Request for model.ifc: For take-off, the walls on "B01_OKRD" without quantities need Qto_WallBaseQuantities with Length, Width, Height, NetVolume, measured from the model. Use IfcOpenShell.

First a look at what the model holds.

```python
import ifcopenshell
import ifcopenshell.util.element
import ifcopenshell.util.unit

model = ifcopenshell.open("model.ifc")
print(model.schema)
for unit_type in ("LENGTHUNIT", "AREAUNIT", "VOLUMEUNIT"):
    print(unit_type, ifcopenshell.util.unit.calculate_unit_scale(model, unit_type))
storey = next(s for s in model.by_type("IfcBuildingStorey") if s.Name == "B01_OKRD")
walls = [e for e in ifcopenshell.util.element.get_decomposition(storey) if e.is_a("IfcWall")]
for e in sorted(walls, key=lambda e: e.id()):
    print(e.id(), e.is_a(), e.Name, list(ifcopenshell.util.element.get_psets(e, qtos_only=True)), sep=" | ")
```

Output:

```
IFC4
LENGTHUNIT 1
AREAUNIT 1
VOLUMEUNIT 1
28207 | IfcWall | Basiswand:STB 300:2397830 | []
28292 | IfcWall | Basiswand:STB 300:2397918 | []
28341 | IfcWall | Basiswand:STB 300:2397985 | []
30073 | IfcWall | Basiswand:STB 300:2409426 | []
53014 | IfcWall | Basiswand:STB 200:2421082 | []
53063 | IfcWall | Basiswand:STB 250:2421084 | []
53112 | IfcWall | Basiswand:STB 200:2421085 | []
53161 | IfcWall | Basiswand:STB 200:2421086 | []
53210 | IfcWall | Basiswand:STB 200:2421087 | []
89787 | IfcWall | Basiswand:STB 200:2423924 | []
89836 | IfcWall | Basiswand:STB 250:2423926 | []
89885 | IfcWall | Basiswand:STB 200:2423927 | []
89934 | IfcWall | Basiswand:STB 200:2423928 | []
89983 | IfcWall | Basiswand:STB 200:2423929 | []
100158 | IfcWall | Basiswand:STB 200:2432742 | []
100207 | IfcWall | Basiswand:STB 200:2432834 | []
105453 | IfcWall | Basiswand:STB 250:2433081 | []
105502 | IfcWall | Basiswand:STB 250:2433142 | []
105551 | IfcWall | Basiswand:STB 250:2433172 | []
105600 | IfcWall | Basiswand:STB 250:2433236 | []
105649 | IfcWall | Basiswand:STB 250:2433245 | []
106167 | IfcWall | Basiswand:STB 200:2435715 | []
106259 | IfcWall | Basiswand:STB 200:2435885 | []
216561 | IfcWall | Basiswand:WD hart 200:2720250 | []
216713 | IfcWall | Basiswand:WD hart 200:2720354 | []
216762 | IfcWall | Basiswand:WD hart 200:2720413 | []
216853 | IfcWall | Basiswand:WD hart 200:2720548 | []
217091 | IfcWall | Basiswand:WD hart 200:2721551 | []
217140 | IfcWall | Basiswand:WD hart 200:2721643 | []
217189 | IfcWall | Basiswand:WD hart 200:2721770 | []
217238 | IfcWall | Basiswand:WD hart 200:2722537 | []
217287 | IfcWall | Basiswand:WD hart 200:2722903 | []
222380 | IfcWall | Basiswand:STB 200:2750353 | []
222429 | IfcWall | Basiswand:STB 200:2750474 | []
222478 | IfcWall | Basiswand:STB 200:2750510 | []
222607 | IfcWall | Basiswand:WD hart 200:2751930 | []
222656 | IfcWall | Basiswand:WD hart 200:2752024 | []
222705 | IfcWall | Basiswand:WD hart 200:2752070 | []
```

```python
import ifcopenshell
import ifcopenshell.api.pset
import ifcopenshell.geom
import ifcopenshell.util.element
import ifcopenshell.util.shape
import ifcopenshell.util.unit

model = ifcopenshell.open("model.ifc")
unit_scale = ifcopenshell.util.unit.calculate_unit_scale(model)
volume_scale = ifcopenshell.util.unit.calculate_unit_scale(model, "VOLUMEUNIT")
settings = ifcopenshell.geom.settings()

storey = next(s for s in model.by_type("IfcBuildingStorey") if s.Name == "B01_OKRD")
walls = [e for e in ifcopenshell.util.element.get_decomposition(storey) if e.is_a("IfcWall")]

for e in sorted(walls, key=lambda e: e.id()):
    if ifcopenshell.util.element.get_psets(e, qtos_only=True, should_inherit=False):
        continue
    # Geometry comes back in metres, in the element's own axes.
    shape = ifcopenshell.geom.create_shape(settings, e)
    values = {
        "Length": ifcopenshell.util.shape.get_x(shape.geometry) / unit_scale,
        "Width": ifcopenshell.util.shape.get_y(shape.geometry) / unit_scale,
        "Height": ifcopenshell.util.shape.get_z(shape.geometry) / unit_scale,
        "NetVolume": ifcopenshell.util.shape.get_volume(shape.geometry) / volume_scale,
    }
    qto = ifcopenshell.api.pset.add_qto(model, product=e, name="Qto_WallBaseQuantities")
    ifcopenshell.api.pset.edit_qto(model, qto=qto, properties=values)
    print(e.id(), {k: round(v, 3) for k, v in values.items()})

model.write("model-out.ifc")
```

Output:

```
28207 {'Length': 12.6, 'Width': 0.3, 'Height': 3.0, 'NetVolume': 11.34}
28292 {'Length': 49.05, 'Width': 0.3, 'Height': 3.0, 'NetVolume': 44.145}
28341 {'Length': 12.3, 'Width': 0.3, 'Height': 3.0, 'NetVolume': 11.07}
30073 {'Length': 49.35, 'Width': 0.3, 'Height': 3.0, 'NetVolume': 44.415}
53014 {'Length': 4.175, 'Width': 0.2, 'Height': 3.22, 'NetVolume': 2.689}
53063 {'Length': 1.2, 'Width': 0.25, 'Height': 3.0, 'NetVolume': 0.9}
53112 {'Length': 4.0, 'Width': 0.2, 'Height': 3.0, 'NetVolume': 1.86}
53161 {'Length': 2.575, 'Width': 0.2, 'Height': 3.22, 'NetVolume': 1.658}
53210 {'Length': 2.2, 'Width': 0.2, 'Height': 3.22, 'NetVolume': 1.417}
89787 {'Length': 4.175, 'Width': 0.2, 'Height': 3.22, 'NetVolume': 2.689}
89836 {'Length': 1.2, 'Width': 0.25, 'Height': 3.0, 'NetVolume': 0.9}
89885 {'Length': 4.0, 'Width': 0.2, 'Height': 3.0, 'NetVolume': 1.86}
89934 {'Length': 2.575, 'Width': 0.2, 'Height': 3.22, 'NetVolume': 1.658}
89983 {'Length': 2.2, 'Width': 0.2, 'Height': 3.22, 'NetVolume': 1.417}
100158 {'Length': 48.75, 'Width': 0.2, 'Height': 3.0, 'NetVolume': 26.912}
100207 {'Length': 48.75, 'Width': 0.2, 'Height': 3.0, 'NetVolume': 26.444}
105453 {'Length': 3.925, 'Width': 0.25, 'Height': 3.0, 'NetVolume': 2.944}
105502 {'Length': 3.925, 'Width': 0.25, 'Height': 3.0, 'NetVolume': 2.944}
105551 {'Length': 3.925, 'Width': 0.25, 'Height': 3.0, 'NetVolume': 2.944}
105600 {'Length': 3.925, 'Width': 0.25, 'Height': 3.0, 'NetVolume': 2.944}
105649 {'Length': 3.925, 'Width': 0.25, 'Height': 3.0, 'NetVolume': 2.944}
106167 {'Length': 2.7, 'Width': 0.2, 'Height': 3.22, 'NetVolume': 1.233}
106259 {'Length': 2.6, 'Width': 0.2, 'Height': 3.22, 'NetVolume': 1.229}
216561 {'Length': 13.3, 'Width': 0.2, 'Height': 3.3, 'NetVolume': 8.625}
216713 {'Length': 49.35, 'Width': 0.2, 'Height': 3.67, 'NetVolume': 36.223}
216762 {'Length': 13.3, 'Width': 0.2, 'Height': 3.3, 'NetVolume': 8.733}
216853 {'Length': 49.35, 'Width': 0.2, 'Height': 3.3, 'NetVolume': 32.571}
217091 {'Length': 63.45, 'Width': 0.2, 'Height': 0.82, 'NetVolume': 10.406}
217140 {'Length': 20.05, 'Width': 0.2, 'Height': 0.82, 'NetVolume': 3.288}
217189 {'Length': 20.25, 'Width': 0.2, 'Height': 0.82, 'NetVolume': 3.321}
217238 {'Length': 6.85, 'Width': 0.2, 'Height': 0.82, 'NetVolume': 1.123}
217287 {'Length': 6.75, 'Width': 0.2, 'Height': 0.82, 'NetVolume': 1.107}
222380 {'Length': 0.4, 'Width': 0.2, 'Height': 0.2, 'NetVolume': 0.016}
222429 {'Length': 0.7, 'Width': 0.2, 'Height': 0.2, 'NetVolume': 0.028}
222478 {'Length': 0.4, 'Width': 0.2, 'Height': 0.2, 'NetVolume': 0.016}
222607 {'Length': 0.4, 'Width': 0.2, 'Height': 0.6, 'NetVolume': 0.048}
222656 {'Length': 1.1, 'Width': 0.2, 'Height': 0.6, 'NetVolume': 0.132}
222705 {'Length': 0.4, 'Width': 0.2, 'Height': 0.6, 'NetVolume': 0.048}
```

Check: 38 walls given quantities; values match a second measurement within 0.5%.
